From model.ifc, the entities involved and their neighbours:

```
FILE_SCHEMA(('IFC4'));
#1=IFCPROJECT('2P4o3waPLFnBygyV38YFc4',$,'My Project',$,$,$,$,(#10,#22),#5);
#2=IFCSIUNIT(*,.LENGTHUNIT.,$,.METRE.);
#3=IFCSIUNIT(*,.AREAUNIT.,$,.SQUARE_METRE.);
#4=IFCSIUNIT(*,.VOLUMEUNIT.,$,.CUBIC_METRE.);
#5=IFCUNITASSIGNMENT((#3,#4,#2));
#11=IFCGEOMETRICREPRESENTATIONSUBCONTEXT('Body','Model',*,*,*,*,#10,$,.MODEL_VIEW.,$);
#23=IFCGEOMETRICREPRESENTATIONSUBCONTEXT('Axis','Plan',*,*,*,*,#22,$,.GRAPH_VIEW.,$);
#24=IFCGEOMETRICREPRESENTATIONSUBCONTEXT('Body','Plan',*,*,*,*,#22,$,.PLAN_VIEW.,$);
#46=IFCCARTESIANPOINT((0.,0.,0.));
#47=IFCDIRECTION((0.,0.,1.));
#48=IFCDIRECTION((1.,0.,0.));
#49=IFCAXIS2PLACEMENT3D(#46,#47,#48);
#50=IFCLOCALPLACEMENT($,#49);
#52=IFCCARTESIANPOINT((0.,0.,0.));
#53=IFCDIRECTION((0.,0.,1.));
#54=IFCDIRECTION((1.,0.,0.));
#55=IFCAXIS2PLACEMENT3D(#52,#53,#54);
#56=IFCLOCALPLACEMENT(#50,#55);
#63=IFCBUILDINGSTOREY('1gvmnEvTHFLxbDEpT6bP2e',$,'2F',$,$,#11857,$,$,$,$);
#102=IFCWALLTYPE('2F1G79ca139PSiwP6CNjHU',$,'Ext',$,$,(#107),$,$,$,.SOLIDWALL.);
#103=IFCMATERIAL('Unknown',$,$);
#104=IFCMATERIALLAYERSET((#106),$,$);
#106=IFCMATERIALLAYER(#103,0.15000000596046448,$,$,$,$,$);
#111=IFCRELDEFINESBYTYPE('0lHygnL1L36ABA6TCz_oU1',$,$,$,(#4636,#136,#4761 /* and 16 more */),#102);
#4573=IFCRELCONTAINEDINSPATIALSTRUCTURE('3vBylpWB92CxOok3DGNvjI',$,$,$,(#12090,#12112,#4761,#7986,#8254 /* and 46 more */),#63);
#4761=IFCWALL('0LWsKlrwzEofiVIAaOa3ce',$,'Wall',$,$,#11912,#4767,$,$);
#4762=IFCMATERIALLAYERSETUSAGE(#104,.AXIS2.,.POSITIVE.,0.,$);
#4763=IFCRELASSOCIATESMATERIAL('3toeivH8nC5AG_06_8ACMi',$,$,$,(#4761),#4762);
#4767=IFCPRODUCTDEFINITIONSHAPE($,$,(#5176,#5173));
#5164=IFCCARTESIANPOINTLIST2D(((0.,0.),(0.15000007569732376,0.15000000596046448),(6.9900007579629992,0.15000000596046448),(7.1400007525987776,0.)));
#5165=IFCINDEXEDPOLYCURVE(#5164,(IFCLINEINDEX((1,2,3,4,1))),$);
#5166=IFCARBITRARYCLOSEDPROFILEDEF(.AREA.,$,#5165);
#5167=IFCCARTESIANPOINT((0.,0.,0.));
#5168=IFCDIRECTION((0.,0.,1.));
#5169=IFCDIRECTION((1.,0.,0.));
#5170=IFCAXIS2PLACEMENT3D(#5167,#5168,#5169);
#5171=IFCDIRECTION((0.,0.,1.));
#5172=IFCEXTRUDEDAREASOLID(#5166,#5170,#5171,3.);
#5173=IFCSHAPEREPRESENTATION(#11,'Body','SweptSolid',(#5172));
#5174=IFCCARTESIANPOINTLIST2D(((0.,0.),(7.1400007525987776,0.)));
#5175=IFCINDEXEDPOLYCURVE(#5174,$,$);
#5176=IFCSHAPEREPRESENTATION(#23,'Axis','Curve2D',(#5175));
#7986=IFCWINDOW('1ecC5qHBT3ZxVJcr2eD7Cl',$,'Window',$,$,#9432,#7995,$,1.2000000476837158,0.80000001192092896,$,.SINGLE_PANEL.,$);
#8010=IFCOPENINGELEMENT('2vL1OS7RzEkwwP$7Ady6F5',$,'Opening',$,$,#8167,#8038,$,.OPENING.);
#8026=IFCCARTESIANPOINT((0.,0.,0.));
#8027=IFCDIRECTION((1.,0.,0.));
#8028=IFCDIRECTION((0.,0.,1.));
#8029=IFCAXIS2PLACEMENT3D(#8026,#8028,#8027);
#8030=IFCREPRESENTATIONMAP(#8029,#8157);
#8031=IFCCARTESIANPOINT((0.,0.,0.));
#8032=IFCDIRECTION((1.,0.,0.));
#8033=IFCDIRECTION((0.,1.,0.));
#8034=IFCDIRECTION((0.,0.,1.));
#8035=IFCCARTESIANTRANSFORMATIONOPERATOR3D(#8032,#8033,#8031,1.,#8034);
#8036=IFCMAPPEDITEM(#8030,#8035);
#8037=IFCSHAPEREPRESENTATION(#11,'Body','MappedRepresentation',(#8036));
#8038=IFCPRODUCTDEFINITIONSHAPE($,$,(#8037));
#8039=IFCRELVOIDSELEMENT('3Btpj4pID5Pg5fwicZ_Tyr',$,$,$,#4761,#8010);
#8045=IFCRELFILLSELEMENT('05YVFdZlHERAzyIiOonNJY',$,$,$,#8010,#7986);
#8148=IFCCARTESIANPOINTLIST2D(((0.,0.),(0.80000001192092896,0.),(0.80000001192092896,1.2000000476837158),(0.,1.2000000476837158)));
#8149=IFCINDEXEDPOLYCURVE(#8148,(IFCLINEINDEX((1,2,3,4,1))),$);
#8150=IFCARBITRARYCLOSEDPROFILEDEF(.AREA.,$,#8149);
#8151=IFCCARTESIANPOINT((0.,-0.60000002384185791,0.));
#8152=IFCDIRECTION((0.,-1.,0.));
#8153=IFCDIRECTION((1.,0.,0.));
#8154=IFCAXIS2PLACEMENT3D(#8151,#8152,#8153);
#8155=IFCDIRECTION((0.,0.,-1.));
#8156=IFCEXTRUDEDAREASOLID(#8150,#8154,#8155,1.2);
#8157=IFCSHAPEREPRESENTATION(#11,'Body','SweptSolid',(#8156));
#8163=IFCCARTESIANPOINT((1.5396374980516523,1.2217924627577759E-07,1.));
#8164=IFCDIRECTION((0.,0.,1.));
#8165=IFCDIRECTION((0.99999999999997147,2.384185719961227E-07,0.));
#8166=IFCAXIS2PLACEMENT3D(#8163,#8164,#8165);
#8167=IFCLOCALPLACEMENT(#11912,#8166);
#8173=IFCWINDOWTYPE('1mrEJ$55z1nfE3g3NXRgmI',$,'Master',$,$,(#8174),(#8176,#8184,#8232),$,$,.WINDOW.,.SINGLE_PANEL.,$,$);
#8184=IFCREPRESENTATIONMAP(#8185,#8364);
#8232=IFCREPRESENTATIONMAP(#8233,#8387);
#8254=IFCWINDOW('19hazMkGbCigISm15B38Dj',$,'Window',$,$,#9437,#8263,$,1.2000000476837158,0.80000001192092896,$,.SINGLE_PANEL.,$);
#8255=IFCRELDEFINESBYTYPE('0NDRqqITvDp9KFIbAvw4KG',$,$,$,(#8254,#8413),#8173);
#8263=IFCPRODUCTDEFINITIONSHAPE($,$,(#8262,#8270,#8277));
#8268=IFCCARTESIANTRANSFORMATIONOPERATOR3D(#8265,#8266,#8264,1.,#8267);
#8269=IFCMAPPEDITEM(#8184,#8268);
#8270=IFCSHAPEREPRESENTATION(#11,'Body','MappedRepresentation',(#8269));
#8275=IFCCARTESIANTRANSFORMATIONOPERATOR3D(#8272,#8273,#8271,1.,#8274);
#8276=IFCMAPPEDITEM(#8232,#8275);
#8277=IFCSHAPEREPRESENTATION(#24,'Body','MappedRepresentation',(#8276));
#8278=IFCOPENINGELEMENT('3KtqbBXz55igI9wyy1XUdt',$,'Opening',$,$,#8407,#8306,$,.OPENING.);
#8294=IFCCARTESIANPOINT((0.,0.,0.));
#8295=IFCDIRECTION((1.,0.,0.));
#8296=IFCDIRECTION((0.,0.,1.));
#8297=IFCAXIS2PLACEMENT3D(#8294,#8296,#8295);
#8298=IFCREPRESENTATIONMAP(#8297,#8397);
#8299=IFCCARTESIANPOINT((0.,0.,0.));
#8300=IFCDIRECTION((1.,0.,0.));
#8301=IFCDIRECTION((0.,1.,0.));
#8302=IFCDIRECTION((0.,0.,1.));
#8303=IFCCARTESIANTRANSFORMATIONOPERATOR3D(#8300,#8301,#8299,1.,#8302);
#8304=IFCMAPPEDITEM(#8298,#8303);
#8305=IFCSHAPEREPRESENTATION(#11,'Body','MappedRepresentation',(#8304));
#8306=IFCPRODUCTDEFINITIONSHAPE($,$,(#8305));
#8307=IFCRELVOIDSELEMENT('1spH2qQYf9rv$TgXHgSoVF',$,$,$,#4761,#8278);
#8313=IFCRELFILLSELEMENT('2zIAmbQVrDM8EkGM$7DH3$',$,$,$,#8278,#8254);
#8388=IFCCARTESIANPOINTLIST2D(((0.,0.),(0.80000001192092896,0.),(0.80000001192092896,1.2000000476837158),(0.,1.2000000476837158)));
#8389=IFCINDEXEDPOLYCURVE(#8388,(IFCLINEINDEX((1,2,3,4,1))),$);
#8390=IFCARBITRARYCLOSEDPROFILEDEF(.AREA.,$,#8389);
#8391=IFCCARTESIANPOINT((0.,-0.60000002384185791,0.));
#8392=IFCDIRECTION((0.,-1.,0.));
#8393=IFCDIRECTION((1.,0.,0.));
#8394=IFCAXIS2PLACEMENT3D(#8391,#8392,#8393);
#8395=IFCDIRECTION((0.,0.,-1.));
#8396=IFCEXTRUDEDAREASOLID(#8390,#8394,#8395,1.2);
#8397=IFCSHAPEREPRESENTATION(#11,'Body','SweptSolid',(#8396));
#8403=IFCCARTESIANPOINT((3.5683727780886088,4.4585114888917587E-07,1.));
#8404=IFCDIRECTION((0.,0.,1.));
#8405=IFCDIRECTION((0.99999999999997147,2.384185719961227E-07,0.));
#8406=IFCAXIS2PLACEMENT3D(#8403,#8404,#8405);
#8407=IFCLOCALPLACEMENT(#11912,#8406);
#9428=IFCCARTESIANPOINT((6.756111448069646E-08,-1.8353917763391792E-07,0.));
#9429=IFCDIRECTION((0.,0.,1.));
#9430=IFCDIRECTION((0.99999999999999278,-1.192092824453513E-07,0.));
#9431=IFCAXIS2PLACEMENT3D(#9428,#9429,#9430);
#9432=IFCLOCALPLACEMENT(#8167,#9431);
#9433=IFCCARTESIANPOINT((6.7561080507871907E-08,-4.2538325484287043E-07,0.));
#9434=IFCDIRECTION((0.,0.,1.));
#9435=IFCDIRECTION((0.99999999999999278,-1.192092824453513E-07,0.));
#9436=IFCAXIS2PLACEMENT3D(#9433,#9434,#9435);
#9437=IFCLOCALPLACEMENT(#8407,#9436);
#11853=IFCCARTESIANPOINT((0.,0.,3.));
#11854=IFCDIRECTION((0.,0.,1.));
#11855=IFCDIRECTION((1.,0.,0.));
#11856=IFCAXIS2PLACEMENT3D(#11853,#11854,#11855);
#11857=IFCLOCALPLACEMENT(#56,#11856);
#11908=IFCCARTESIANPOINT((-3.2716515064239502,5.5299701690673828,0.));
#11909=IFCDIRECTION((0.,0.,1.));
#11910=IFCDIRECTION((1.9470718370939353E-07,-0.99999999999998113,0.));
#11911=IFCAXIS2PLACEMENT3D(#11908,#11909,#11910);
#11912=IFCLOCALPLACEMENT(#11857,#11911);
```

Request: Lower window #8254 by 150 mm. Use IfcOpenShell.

```python
import numpy as np
import ifcopenshell
import ifcopenshell.api.geometry
import ifcopenshell.util.placement
import ifcopenshell.util.unit

model = ifcopenshell.open("model.ifc")
unit_scale = ifcopenshell.util.unit.calculate_unit_scale(model)

window = model.by_guid("19hazMkGbCigISm15B38Dj")
opening = window.FillsVoids[0].RelatingOpeningElement
dz = -0.15 / unit_scale

shift = np.array([0.0, 0.0, dz])
# The window is placed relative to its opening, so it follows when the opening moves.
matrix = ifcopenshell.util.placement.get_local_placement(opening.ObjectPlacement)
matrix[:3, 3] += shift
ifcopenshell.api.geometry.edit_object_placement(
    model, product=opening, matrix=matrix, is_si=False, should_transform_children=True
)

print(f"moved by {dz * unit_scale:+.3f} m")

model.write("model-out.ifc")
```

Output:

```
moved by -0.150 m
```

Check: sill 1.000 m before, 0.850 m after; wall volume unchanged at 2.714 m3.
